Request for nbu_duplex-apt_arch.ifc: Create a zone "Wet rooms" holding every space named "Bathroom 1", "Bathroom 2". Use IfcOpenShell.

First a look at what the model holds.

```python
import ifcopenshell

model = ifcopenshell.open("nbu_duplex-apt_arch.ifc")
print(model.schema)
seen = {}
for space in model.by_type("IfcSpace"):
    seen[space.LongName] = seen.get(space.LongName, 0) + 1
for name, count in sorted(seen.items(), key=str):
    print(count, "x", name)
print("zones:", [z.Name for z in model.by_type("IfcZone")][:20])
```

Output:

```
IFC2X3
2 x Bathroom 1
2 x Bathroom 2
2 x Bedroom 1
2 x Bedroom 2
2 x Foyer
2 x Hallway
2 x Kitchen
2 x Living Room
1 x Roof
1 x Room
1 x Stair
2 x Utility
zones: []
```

```python
import ifcopenshell
import ifcopenshell.api.group
import ifcopenshell.api.root

model = ifcopenshell.open("nbu_duplex-apt_arch.ifc")

names = {"Bathroom 1", "Bathroom 2"}
spaces = [s for s in model.by_type("IfcSpace") if s.LongName in names]

zone = ifcopenshell.api.root.create_entity(model, ifc_class="IfcZone", name="Wet rooms")
ifcopenshell.api.group.assign_group(model, products=spaces, group=zone)
print(len(spaces), "spaces in", zone.Name)

model.write("nbu_duplex-apt_arch-out.ifc")
```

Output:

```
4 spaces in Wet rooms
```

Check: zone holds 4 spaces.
